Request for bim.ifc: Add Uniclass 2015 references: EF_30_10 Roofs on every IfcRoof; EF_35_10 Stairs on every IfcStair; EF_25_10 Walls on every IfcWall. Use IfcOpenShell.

First a look at what the model holds.

```python
import ifcopenshell

model = ifcopenshell.open("bim.ifc")
print(model.schema)
print("classifications:", [c.Name for c in model.by_type("IfcClassification")])
for ifc_class in ("IfcDoor", "IfcRoof", "IfcStair", "IfcWall", "IfcWindow"):
    print(ifc_class, len(model.by_type(ifc_class)))
```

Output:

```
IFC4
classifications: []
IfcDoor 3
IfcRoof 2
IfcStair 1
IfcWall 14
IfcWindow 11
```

```python
import ifcopenshell
import ifcopenshell.api.classification

model = ifcopenshell.open("bim.ifc")

system = ifcopenshell.api.classification.add_classification(model, classification="Uniclass 2015")

codes = {
    "IfcRoof": ("EF_30_10", "Roofs"),
    "IfcStair": ("EF_35_10", "Stairs"),
    "IfcWall": ("EF_25_10", "Walls"),
}
for ifc_class, (code, name) in codes.items():
    products = model.by_type(ifc_class)
    ifcopenshell.api.classification.add_reference(
        model, products=products, classification=system, identification=code, name=name
    )
    print(code, len(products))

model.write("bim_edited.ifc")
```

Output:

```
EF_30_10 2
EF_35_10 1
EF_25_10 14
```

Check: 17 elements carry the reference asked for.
